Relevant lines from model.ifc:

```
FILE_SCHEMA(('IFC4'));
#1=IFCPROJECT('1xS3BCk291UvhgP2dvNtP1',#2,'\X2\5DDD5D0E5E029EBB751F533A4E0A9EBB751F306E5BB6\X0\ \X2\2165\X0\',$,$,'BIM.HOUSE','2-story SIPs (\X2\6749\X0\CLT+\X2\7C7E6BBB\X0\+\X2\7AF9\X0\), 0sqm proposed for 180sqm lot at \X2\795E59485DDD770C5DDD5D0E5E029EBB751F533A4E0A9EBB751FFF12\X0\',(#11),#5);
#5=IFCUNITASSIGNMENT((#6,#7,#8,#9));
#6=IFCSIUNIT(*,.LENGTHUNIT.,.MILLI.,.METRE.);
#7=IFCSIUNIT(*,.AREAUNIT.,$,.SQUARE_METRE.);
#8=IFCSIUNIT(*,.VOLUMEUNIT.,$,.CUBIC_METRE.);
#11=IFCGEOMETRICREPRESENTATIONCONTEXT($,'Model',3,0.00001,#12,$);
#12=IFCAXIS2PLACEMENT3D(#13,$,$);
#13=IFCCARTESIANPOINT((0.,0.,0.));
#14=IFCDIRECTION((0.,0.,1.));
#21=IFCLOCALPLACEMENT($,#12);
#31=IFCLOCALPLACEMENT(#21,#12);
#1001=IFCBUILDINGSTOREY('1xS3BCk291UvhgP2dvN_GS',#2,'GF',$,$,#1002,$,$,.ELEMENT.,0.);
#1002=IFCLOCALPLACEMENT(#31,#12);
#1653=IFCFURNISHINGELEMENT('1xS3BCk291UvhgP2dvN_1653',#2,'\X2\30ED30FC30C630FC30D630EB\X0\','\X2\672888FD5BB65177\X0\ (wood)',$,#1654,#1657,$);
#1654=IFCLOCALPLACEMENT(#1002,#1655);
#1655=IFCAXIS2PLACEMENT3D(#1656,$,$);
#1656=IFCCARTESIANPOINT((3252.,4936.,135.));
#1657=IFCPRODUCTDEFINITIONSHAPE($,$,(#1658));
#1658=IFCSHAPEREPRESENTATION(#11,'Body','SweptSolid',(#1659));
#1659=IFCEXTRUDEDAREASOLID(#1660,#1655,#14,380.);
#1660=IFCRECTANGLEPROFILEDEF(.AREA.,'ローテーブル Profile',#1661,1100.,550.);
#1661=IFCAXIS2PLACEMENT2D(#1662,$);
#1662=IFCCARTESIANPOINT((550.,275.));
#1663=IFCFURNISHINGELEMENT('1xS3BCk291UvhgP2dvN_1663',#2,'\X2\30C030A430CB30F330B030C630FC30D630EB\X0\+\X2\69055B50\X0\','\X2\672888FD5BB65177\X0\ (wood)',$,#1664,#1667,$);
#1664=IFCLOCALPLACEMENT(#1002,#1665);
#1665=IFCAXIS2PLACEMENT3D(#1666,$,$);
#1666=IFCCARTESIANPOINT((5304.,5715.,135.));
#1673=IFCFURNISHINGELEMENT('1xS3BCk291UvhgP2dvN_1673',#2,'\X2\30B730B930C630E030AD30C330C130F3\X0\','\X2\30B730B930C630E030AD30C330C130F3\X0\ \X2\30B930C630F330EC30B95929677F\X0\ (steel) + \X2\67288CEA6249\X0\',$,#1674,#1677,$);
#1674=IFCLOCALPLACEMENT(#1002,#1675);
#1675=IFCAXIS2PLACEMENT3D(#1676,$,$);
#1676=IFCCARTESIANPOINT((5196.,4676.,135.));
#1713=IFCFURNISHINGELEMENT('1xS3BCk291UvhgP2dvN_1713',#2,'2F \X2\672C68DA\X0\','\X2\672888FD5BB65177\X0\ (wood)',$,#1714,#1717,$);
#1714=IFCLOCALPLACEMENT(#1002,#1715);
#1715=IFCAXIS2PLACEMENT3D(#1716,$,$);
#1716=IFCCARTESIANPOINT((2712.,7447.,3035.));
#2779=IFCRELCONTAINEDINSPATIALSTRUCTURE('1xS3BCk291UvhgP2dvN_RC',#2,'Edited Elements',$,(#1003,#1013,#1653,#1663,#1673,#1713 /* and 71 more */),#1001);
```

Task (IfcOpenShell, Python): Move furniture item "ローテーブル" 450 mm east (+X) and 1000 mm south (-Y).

```python
import ifcopenshell
import ifcopenshell.api.geometry
import ifcopenshell.util.placement

model = ifcopenshell.open("model.ifc")

item = model.by_guid("1xS3BCk291UvhgP2dvN_1653")
matrix = ifcopenshell.util.placement.get_local_placement(item.ObjectPlacement)
matrix[0, 3] += 450.0
matrix[1, 3] -= 1000.0
ifcopenshell.api.geometry.edit_object_placement(model, product=item, matrix=matrix, is_si=False)

print(ifcopenshell.util.placement.get_local_placement(item.ObjectPlacement).round(3) + 0.0)

model.write("model-out.ifc")
```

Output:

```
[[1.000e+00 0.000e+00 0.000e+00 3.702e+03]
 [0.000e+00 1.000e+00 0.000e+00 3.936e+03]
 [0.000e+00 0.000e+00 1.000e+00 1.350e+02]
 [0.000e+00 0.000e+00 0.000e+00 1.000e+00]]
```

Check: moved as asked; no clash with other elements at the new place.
